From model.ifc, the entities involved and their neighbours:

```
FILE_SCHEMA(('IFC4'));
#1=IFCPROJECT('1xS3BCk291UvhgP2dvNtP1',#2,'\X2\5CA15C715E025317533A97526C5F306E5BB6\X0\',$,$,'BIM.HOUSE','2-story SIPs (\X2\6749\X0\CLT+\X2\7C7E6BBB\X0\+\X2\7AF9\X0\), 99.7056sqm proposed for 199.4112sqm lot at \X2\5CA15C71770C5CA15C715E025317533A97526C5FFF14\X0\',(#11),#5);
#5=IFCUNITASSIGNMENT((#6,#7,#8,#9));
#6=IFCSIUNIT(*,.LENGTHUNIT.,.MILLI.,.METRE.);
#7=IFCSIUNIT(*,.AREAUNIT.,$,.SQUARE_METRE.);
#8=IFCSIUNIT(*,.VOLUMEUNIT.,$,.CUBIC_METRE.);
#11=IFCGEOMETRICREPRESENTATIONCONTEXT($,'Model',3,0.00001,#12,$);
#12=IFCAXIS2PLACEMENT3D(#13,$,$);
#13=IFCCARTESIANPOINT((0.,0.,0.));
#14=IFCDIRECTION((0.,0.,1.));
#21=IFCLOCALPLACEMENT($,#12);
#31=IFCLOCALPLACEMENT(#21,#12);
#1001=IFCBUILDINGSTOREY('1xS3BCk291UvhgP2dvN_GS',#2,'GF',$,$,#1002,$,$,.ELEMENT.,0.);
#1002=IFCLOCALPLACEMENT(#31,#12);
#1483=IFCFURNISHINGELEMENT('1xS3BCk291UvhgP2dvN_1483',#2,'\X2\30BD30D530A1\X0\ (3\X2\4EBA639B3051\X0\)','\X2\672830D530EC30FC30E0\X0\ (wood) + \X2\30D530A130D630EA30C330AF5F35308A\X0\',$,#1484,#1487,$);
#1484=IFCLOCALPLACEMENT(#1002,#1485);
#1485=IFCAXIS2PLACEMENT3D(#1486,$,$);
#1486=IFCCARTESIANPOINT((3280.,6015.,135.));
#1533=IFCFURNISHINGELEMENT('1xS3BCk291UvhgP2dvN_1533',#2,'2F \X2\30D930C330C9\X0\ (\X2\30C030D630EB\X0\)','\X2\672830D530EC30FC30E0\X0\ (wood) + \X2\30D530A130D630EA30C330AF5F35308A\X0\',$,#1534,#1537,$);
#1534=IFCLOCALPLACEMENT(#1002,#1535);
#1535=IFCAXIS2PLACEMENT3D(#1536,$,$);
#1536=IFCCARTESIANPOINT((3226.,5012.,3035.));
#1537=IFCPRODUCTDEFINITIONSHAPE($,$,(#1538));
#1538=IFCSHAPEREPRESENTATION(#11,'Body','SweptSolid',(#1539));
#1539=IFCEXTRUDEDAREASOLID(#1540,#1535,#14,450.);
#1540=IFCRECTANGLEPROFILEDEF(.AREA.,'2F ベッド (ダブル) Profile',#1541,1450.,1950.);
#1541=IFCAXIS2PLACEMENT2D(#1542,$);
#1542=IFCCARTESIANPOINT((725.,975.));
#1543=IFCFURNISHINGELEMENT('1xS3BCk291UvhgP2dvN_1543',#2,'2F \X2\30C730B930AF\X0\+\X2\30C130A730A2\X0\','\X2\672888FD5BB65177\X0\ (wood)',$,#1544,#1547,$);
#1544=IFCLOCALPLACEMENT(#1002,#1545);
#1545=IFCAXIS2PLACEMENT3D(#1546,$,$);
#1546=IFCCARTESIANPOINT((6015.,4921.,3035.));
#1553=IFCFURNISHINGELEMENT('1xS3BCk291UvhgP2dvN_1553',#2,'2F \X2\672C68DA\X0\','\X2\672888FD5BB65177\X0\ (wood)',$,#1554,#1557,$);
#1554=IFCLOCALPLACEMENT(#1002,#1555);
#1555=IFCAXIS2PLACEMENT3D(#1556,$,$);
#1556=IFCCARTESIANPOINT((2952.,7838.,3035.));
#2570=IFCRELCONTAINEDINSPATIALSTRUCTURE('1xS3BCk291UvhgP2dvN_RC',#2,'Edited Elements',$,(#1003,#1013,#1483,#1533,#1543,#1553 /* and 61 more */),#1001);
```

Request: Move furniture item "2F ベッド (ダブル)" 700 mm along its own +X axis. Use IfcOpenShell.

```python
import ifcopenshell
import ifcopenshell.api.geometry
import ifcopenshell.util.placement
import ifcopenshell.util.unit

model = ifcopenshell.open("model.ifc")
unit_scale = ifcopenshell.util.unit.calculate_unit_scale(model)

item = model.by_guid("1xS3BCk291UvhgP2dvN_1533")
matrix = ifcopenshell.util.placement.get_local_placement(item.ObjectPlacement)
matrix[:3, 3] += matrix[:3, 0] * 0.7 / unit_scale
ifcopenshell.api.geometry.edit_object_placement(model, product=item, matrix=matrix, is_si=False)

print(ifcopenshell.util.placement.get_local_placement(item.ObjectPlacement).round(3) + 0.0)

model.write("model_v2.ifc")
```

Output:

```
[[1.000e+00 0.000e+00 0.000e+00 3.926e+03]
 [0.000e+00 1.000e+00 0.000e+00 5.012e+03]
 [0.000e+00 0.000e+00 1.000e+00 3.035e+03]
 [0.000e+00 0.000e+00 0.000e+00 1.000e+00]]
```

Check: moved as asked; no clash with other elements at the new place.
